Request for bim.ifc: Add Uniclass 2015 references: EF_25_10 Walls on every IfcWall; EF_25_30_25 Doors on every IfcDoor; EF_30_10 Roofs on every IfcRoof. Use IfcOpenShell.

First a look at what the model holds.

```python
import ifcopenshell

model = ifcopenshell.open("bim.ifc")
print(model.schema)
print("classifications:", [c.Name for c in model.by_type("IfcClassification")])
for ifc_class in ("IfcDoor", "IfcRoof", "IfcStair", "IfcWall", "IfcWindow"):
    print(ifc_class, len(model.by_type(ifc_class)))
```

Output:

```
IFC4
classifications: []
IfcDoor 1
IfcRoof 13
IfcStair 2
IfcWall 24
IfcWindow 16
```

```python
import ifcopenshell
import ifcopenshell.api.classification

model = ifcopenshell.open("bim.ifc")

system = ifcopenshell.api.classification.add_classification(model, classification="Uniclass 2015")

codes = {
    "IfcWall": ("EF_25_10", "Walls"),
    "IfcDoor": ("EF_25_30_25", "Doors"),
    "IfcRoof": ("EF_30_10", "Roofs"),
}
for ifc_class, (code, name) in codes.items():
    products = model.by_type(ifc_class)
    ifcopenshell.api.classification.add_reference(
        model, products=products, classification=system, identification=code, name=name
    )
    print(code, len(products))

model.write("bim_edited.ifc")
```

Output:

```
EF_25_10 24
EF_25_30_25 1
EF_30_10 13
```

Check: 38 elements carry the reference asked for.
